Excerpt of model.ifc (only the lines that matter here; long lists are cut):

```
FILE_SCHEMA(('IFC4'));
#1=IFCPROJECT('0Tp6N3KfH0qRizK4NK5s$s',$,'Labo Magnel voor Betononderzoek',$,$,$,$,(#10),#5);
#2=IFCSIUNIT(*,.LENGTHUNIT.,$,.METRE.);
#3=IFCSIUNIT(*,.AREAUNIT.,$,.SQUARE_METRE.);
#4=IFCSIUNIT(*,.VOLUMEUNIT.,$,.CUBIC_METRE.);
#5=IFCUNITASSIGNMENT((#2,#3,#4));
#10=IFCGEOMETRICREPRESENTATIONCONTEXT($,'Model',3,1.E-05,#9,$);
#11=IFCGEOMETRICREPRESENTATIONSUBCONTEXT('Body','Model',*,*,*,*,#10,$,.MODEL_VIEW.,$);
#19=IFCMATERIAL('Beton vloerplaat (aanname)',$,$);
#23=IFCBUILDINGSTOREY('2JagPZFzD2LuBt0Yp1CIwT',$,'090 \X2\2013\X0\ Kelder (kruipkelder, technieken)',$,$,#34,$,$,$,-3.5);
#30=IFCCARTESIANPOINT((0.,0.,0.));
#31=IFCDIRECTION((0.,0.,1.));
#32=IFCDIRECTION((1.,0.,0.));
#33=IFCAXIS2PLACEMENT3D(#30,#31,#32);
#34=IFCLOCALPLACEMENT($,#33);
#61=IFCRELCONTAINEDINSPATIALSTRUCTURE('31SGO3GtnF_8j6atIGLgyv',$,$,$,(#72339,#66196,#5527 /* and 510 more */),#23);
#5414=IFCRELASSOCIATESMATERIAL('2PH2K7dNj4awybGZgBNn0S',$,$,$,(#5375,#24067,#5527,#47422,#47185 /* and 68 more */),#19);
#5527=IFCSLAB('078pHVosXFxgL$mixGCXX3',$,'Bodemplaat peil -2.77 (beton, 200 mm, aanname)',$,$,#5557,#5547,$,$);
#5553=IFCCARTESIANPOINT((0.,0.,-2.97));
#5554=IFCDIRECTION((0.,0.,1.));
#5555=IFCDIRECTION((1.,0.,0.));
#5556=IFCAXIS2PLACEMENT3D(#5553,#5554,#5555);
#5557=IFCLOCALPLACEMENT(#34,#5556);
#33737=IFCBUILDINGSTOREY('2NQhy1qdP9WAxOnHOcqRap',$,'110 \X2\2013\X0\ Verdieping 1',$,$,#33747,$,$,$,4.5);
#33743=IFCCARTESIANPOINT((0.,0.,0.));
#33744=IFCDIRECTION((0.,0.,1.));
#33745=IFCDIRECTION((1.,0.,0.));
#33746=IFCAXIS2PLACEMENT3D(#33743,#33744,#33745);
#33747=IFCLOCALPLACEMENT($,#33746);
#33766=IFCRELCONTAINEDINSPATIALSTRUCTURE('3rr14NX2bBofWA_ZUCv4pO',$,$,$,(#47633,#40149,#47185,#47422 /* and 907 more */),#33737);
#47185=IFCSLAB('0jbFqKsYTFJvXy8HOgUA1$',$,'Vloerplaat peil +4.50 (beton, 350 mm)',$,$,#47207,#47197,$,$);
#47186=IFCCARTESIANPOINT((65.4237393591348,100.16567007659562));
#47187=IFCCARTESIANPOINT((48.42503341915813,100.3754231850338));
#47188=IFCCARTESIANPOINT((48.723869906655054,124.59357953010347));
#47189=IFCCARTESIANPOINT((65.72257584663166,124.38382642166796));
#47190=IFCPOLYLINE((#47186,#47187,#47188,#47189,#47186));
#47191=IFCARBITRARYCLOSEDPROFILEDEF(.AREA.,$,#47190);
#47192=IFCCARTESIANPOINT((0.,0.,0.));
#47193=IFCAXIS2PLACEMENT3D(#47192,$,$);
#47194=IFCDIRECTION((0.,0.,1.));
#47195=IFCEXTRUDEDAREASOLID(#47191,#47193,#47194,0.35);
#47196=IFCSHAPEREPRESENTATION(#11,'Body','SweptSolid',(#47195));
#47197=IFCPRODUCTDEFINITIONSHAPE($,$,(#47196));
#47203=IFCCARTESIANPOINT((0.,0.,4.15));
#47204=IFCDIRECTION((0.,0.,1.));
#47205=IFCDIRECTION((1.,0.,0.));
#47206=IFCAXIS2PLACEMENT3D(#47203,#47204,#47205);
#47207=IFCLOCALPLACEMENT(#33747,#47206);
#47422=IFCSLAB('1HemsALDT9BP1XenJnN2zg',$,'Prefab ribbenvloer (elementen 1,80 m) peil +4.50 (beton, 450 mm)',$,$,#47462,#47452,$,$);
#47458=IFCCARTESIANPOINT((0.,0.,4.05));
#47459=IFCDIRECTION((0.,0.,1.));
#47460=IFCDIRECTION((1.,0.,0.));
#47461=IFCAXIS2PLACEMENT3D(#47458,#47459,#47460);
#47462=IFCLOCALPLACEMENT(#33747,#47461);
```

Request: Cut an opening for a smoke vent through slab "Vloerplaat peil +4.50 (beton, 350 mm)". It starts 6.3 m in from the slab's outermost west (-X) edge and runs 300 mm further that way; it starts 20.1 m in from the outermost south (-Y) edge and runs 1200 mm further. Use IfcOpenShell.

```python
import numpy as np
import ifcopenshell
import ifcopenshell.api.feature
import ifcopenshell.api.geometry
import ifcopenshell.api.root
import ifcopenshell.geom
import ifcopenshell.util.placement
import ifcopenshell.util.representation
import ifcopenshell.util.shape
import ifcopenshell.util.unit

model = ifcopenshell.open("model.ifc")
unit_scale = ifcopenshell.util.unit.calculate_unit_scale(model)
settings = ifcopenshell.geom.settings()


def volume(element):
    """Net volume in cubic metres, openings subtracted."""
    shape = ifcopenshell.geom.create_shape(settings, element)
    return ifcopenshell.util.shape.get_volume(shape.geometry)


slab = model.by_id(47185)
before = volume(slab)

# Extent in the slab's own axes, in metres. The edges named are its -X and -Y sides.
slab_shape = ifcopenshell.geom.create_shape(settings, slab)
vertices = ifcopenshell.util.shape.get_vertices(slab_shape.geometry)
x_min, y_min, bottom = vertices.min(axis=0)
top = vertices[:, 2].max()

opening = ifcopenshell.api.root.create_entity(model, ifc_class="IfcOpeningElement", name="Smoke vent opening", predefined_type="OPENING")
context = ifcopenshell.util.representation.get_context(model, "Model", "Body", "MODEL_VIEW")
width, depth = 0.3, 1.2
outline = [(0.0, 0.0), (width, 0.0), (width, depth), (0.0, depth), (0.0, 0.0)]
# Overshoot both faces by 50 mm so the cut is clean.
shape = ifcopenshell.api.geometry.add_slab_representation(
    model, context=context, depth=top - bottom + 0.1, polyline=outline
)
ifcopenshell.api.geometry.assign_representation(model, product=opening, representation=shape)

matrix = ifcopenshell.util.placement.get_local_placement(slab.ObjectPlacement)
matrix[:, 3] = matrix @ np.append(np.array([x_min + 6.3, y_min + 20.1, bottom - 0.05]) / unit_scale, 1.0)
ifcopenshell.api.geometry.edit_object_placement(model, product=opening, matrix=matrix, is_si=False)
ifcopenshell.api.feature.add_feature(model, feature=opening, element=slab)

after = volume(slab)

print(f"slab volume {before:.3f} -> {after:.3f} m3")

model.write("model-out.ifc")
```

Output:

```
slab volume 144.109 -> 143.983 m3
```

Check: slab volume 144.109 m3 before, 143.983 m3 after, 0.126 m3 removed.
